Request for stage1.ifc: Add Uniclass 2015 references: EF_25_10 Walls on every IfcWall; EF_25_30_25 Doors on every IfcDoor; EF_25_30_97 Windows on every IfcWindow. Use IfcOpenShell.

First a look at what the model holds.

```python
import ifcopenshell

model = ifcopenshell.open("stage1.ifc")
print(model.schema)
print("classifications:", [c.Name for c in model.by_type("IfcClassification")])
for ifc_class in ("IfcDoor", "IfcRoof", "IfcStair", "IfcWall", "IfcWindow"):
    print(ifc_class, len(model.by_type(ifc_class)))
```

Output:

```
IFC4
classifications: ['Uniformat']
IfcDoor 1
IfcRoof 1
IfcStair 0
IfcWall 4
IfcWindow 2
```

```python
import ifcopenshell
import ifcopenshell.api.classification

model = ifcopenshell.open("stage1.ifc")

system = ifcopenshell.api.classification.add_classification(model, classification="Uniclass 2015")

codes = {
    "IfcWall": ("EF_25_10", "Walls"),
    "IfcDoor": ("EF_25_30_25", "Doors"),
    "IfcWindow": ("EF_25_30_97", "Windows"),
}
for ifc_class, (code, name) in codes.items():
    products = model.by_type(ifc_class)
    ifcopenshell.api.classification.add_reference(
        model, products=products, classification=system, identification=code, name=name
    )
    print(code, len(products))

model.write("stage1_edited.ifc")
```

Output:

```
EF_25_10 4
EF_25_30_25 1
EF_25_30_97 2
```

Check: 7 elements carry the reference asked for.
